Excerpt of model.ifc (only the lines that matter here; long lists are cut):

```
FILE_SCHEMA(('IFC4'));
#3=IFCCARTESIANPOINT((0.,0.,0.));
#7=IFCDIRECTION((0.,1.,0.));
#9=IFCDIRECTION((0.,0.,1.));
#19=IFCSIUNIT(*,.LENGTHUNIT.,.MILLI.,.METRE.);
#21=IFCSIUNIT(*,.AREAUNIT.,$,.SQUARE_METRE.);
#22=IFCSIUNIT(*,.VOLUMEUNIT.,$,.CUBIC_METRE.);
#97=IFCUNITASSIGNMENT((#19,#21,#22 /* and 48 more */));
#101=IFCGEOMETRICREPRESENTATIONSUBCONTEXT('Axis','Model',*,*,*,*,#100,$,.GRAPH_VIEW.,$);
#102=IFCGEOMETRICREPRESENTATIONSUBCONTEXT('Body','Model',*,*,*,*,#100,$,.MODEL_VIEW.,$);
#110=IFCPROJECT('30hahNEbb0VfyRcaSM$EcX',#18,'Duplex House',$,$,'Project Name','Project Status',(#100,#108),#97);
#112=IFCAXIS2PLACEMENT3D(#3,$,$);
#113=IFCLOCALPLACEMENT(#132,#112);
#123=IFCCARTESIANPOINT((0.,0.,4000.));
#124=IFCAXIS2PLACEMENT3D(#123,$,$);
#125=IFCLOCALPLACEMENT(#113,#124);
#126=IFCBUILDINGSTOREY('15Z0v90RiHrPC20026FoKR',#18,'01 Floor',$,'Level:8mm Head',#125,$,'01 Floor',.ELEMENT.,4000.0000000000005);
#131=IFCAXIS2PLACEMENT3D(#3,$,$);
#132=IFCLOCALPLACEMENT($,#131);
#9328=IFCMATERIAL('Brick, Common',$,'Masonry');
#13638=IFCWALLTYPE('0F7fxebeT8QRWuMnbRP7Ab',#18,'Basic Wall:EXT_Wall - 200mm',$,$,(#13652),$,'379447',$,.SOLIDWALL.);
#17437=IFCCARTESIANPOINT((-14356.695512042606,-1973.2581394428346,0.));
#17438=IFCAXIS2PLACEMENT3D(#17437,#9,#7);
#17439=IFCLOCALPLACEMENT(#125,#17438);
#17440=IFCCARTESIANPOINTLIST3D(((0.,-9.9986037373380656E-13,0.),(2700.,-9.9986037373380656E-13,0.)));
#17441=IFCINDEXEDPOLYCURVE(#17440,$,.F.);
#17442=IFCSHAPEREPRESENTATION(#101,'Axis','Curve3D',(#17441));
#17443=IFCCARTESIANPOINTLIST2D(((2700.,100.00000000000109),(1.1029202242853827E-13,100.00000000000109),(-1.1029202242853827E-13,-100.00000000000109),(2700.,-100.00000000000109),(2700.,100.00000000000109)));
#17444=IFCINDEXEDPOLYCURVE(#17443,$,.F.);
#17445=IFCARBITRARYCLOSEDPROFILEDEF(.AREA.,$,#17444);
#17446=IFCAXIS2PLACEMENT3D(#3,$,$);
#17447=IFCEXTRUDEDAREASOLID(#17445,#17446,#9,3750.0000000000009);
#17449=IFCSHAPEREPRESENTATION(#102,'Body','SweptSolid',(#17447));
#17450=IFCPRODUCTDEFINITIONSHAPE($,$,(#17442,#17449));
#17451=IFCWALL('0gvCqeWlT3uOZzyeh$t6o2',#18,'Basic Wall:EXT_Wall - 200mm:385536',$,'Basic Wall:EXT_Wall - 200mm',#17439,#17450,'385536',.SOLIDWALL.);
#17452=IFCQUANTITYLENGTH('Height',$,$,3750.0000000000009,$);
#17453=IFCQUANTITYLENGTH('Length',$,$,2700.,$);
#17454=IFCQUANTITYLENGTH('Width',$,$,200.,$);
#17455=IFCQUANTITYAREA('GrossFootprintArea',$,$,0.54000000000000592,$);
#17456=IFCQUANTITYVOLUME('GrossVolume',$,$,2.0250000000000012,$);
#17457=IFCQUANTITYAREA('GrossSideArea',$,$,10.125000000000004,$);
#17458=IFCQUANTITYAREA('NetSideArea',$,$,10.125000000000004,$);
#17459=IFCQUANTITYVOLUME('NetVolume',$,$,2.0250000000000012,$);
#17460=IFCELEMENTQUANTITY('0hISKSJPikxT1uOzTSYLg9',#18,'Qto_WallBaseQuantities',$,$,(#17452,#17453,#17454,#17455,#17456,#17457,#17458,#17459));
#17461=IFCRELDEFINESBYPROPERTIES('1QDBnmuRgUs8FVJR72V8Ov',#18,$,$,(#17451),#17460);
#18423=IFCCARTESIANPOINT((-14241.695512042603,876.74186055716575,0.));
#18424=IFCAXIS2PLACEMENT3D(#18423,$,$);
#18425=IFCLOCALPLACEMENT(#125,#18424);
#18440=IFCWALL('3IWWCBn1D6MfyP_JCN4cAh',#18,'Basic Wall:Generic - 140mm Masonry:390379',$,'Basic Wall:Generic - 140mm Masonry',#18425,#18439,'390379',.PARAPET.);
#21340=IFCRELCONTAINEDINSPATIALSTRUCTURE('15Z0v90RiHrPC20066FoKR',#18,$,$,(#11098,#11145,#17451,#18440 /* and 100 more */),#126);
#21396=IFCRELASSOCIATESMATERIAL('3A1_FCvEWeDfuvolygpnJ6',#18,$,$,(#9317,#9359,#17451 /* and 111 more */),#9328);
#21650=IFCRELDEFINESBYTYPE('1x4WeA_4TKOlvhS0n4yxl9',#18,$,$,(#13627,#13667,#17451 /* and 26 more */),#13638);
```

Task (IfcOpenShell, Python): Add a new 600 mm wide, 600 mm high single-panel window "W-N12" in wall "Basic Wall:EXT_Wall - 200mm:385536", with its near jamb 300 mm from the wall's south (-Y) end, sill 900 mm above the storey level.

```python
import numpy as np
import ifcopenshell
import ifcopenshell.api.feature
import ifcopenshell.api.geometry
import ifcopenshell.api.pset
import ifcopenshell.api.root
import ifcopenshell.api.spatial
import ifcopenshell.geom
import ifcopenshell.util.element
import ifcopenshell.util.placement
import ifcopenshell.util.representation
import ifcopenshell.util.shape
import ifcopenshell.util.unit

model = ifcopenshell.open("model.ifc")
unit_scale = ifcopenshell.util.unit.calculate_unit_scale(model)
area_scale = ifcopenshell.util.unit.calculate_unit_scale(model, "AREAUNIT")
volume_scale = ifcopenshell.util.unit.calculate_unit_scale(model, "VOLUMEUNIT")
settings = ifcopenshell.geom.settings()


def volume(element):
    """Net volume in cubic metres, openings subtracted."""
    shape = ifcopenshell.geom.create_shape(settings, element)
    return ifcopenshell.util.shape.get_volume(shape.geometry)


wall = model.by_id(17451)
storey = ifcopenshell.util.element.get_container(wall, ifc_class="IfcBuildingStorey")
context = ifcopenshell.util.representation.get_context(model, "Model", "Body", "MODEL_VIEW")
before = volume(wall)

width, height, from_end, sill = 0.6, 0.6, 0.3, 0.9  # metres

# The wall runs along its own X axis, and the end named is its -X end.
wall_shape = ifcopenshell.geom.create_shape(settings, wall)
x, y, z = ifcopenshell.util.shape.get_vertices(wall_shape.geometry).T
start = x.min() + from_end
face, thickness = float(y.min()), float(y.max() - y.min())
wall_matrix = ifcopenshell.util.placement.get_local_placement(wall.ObjectPlacement)
level = ifcopenshell.util.placement.get_local_placement(storey.ObjectPlacement)[2, 3]


def in_wall(x, y):
    """Placement at x, y metres in the wall's axes, at sill height."""
    matrix = wall_matrix.copy()
    matrix[:, 3] = wall_matrix @ np.array([x / unit_scale, y / unit_scale, 0.0, 1.0])
    matrix[2, 3] = level + sill / unit_scale
    return matrix


# Opening: a box that overshoots both wall faces by 50 mm.
opening = ifcopenshell.api.root.create_entity(model, ifc_class="IfcOpeningElement", predefined_type="OPENING")
box = ifcopenshell.api.geometry.add_wall_representation(
    model, context=context, length=width, height=height, thickness=thickness + 0.1
)
ifcopenshell.api.geometry.assign_representation(model, product=opening, representation=box)
ifcopenshell.api.geometry.edit_object_placement(model, product=opening, matrix=in_wall(start, face - 0.05), is_si=False)
ifcopenshell.api.feature.add_feature(model, feature=opening, element=wall)

window = ifcopenshell.api.root.create_entity(model, ifc_class="IfcWindow", name="W-N12", predefined_type="WINDOW")
window.OverallWidth, window.OverallHeight = width / unit_scale, height / unit_scale
window.PartitioningType = "SINGLE_PANEL"
body = ifcopenshell.api.geometry.add_window_representation(
    model,
    context=context,
    overall_width=window.OverallWidth,
    overall_height=window.OverallHeight,
    partition_type="SINGLE_PANEL",
)
ifcopenshell.api.geometry.assign_representation(model, product=window, representation=body)
ifcopenshell.api.spatial.assign_container(model, products=[window], relating_structure=storey)
ifcopenshell.api.feature.add_filling(model, opening=opening, element=window)

# Centre the window in the wall's thickness.
ifcopenshell.api.geometry.edit_object_placement(model, product=window, matrix=in_wall(start, face), is_si=False)
window_shape = ifcopenshell.geom.create_shape(settings, window)
depth = ifcopenshell.util.shape.get_vertices(window_shape.geometry)[:, 1]
offset = face + thickness / 2 - (depth.min() + depth.max()) / 2
ifcopenshell.api.geometry.edit_object_placement(model, product=window, matrix=in_wall(start, offset), is_si=False)

after = volume(wall)

# Update the wall's stored quantities.
qto = model.by_id(ifcopenshell.util.element.get_pset(wall, "Qto_WallBaseQuantities", should_inherit=False)["id"])
ifcopenshell.api.pset.edit_qto(model, qto=qto, properties={
    "NetSideArea": after / thickness / area_scale,
    "NetVolume": after / volume_scale,
})

print(f"wall volume {before:.3f} -> {after:.3f} m3")

model.write("model_edited.ifc")
```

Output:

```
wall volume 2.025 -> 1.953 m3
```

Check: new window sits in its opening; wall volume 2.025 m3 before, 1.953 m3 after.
